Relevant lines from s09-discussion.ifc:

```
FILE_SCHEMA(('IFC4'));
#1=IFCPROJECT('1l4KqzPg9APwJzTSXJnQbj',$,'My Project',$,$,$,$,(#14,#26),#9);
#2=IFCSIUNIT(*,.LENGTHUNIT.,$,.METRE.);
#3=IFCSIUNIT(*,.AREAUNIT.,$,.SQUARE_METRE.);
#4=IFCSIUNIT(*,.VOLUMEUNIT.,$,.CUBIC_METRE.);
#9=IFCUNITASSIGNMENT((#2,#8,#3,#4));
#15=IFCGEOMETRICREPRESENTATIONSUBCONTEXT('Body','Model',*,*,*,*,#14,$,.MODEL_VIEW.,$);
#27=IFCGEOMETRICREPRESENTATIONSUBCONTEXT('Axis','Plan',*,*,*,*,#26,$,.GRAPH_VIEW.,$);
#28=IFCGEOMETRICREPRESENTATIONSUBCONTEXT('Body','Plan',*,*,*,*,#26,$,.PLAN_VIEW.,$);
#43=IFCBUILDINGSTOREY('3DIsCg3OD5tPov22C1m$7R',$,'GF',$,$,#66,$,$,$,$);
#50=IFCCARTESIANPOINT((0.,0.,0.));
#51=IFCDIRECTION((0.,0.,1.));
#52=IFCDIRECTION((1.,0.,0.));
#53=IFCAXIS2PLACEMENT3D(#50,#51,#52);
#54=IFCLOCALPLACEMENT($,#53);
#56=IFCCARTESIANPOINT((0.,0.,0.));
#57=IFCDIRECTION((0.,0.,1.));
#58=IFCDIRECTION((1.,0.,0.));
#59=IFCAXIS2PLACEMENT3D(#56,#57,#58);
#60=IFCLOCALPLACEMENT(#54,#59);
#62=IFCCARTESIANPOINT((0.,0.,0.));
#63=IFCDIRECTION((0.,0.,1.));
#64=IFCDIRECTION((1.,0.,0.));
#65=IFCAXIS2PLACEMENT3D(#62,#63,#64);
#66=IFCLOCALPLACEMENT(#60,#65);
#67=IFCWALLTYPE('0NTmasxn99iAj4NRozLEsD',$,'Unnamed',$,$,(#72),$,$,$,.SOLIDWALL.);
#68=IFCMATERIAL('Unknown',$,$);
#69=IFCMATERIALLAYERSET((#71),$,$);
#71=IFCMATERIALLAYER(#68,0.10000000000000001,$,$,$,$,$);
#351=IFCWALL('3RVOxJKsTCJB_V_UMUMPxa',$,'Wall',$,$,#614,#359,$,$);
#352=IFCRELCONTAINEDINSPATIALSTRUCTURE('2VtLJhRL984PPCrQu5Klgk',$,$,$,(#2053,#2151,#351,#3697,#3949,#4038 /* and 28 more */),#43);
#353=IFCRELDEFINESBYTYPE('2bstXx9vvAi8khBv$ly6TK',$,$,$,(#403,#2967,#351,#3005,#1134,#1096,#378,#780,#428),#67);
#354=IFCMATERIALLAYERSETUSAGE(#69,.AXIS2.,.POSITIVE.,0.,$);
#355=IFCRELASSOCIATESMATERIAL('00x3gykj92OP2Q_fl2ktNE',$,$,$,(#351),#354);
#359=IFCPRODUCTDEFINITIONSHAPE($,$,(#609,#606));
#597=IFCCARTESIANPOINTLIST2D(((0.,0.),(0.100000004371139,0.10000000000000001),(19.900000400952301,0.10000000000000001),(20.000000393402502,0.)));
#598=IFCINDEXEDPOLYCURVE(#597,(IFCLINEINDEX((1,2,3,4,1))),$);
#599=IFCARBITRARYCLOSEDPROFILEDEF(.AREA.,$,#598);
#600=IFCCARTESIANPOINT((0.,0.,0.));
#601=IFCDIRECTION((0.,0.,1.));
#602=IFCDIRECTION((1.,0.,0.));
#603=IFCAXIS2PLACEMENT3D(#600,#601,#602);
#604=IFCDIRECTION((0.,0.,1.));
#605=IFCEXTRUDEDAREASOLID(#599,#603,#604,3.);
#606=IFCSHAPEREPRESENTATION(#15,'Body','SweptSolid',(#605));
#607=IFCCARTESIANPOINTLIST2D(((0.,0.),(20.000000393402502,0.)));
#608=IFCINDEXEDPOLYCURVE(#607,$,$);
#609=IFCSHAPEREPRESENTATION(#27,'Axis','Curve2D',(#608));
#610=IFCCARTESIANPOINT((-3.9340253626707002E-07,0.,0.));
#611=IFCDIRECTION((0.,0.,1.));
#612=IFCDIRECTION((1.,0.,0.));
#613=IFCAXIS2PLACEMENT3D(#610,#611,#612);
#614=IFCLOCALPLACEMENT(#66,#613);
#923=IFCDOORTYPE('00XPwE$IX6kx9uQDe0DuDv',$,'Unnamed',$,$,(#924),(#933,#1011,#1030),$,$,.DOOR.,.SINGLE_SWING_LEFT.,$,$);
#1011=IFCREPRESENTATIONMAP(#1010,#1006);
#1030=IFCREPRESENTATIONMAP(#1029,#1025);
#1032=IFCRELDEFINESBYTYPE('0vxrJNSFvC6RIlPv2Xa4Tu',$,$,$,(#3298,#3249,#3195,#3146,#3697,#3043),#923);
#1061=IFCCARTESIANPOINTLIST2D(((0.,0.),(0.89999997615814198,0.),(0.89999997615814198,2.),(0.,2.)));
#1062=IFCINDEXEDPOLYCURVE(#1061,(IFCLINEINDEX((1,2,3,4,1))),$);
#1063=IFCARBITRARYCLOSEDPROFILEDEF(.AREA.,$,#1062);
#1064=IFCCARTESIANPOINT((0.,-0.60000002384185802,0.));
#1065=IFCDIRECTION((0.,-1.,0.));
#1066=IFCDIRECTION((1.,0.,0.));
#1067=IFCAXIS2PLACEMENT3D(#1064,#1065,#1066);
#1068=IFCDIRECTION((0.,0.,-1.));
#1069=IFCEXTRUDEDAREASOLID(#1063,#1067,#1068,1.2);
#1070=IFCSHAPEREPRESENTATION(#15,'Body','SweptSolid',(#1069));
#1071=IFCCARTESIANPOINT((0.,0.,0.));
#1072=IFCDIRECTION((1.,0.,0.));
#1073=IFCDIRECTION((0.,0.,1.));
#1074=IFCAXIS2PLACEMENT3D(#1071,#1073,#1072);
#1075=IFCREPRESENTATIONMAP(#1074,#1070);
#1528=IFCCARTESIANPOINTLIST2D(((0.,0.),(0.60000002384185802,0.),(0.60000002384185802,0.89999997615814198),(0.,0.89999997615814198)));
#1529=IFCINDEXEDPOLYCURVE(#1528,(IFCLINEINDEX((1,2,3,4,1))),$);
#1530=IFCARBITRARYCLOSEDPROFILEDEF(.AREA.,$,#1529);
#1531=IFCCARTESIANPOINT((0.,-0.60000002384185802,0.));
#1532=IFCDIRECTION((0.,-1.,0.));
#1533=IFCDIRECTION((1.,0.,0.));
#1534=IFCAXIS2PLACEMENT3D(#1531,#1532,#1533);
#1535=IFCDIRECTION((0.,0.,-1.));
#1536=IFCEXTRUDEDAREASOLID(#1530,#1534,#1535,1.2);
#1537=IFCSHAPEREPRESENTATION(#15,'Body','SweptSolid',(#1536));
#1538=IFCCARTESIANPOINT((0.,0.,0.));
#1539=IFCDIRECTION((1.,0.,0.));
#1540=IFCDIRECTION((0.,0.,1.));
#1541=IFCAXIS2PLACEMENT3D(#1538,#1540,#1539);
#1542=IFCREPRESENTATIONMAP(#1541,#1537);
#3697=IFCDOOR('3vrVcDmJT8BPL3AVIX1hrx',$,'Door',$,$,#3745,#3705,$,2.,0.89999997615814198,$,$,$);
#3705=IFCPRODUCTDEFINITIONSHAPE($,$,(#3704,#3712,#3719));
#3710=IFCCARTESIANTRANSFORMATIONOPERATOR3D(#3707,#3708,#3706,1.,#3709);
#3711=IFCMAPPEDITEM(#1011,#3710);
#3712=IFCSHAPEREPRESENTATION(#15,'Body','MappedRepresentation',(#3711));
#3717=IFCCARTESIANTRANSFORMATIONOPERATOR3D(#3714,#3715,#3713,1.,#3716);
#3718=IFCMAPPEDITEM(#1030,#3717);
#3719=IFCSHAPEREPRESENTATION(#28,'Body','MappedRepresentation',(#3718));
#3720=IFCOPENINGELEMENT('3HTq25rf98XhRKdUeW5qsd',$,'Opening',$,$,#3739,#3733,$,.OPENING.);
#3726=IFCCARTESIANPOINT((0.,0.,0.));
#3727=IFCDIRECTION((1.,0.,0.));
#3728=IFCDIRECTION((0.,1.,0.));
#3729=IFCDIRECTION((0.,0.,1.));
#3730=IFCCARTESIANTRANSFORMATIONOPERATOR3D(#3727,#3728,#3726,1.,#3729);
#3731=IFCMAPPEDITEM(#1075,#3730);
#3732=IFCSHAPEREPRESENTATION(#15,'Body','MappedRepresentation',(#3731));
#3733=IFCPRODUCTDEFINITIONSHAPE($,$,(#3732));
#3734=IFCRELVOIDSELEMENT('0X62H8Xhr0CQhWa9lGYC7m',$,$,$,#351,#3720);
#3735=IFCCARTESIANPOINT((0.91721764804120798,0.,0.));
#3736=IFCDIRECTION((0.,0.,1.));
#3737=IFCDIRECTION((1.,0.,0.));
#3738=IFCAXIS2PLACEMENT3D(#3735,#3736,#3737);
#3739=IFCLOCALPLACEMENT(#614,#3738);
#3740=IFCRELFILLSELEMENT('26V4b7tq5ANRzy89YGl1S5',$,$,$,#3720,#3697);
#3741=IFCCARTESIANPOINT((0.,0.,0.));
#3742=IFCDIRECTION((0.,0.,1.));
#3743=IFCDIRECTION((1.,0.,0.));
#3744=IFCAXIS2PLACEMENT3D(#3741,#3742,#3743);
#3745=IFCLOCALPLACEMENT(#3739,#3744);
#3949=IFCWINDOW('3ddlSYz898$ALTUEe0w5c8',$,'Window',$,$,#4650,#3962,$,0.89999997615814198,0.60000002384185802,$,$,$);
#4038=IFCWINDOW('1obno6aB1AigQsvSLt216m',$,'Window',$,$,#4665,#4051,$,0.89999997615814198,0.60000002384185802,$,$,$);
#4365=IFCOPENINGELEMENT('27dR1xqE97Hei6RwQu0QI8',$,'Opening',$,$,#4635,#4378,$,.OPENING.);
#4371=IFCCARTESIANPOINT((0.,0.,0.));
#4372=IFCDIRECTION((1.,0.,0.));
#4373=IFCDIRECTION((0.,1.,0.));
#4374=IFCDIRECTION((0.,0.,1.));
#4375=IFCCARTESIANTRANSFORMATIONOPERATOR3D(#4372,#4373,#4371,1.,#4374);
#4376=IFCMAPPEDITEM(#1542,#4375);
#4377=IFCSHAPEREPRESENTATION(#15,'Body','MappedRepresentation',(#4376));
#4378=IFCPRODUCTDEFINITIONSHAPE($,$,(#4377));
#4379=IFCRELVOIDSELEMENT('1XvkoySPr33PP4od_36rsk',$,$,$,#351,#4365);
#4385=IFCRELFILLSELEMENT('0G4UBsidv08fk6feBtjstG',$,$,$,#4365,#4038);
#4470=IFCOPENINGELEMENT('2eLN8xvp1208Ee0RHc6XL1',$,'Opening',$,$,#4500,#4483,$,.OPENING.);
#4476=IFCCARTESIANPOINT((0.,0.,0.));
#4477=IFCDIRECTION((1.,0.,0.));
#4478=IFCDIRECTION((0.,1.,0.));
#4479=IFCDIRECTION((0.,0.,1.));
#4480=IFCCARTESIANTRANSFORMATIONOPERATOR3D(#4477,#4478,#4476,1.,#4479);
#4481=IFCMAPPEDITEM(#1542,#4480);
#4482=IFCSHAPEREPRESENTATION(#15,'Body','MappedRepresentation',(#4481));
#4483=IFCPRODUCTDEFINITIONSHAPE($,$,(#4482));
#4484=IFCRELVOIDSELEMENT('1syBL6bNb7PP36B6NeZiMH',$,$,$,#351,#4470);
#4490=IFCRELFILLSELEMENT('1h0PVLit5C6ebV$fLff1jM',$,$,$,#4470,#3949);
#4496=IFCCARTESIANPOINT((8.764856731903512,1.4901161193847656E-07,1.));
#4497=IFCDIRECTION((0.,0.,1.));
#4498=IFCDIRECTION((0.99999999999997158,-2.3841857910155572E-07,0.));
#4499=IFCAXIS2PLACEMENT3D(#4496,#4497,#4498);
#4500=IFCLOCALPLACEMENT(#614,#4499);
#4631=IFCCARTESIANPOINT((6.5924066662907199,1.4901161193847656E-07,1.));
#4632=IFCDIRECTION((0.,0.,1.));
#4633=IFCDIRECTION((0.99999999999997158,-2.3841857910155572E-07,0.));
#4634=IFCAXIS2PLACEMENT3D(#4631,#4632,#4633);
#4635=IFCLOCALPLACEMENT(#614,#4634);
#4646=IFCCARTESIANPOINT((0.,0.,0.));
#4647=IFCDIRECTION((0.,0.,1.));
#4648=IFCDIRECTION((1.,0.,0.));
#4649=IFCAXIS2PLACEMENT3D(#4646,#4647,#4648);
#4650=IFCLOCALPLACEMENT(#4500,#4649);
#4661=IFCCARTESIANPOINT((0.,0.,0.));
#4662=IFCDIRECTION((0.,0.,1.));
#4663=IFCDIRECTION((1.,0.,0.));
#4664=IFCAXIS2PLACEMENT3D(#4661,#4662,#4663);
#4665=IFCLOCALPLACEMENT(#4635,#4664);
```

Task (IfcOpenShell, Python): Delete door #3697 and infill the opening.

```python
import ifcopenshell
import ifcopenshell.api.feature
import ifcopenshell.api.root
import ifcopenshell.geom
import ifcopenshell.util.shape

model = ifcopenshell.open("s09-discussion.ifc")
settings = ifcopenshell.geom.settings()


def volume(element):
    """Net volume in cubic metres, openings subtracted."""
    shape = ifcopenshell.geom.create_shape(settings, element)
    return ifcopenshell.util.shape.get_volume(shape.geometry)


door = model.by_guid("3vrVcDmJT8BPL3AVIX1hrx")
opening = door.FillsVoids[0].RelatingOpeningElement
wall = opening.VoidsElements[0].RelatingBuildingElement
before = volume(wall)

ifcopenshell.api.root.remove_product(model, product=door)
ifcopenshell.api.feature.remove_feature(model, feature=opening)

after = volume(wall)

print(f"wall volume {before:.3f} -> {after:.3f} m3")

model.write("s09-discussion-out.ifc")
```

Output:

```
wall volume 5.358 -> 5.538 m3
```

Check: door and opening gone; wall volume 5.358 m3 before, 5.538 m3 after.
